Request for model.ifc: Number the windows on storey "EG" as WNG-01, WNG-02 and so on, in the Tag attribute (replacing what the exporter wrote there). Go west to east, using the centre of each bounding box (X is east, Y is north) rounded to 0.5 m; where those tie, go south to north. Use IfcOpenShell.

First a look at what the model holds.

```python
import ifcopenshell
import ifcopenshell.util.element
import ifcopenshell.util.placement

model = ifcopenshell.open("model.ifc")
print(model.schema)
storey = next(s for s in model.by_type("IfcBuildingStorey") if s.Name == "EG")
windows = [e for e in ifcopenshell.util.element.get_decomposition(storey) if e.is_a("IfcWindow")]
for e in sorted(windows, key=lambda e: e.id()):
    origin = ifcopenshell.util.placement.get_local_placement(e.ObjectPlacement)[:3, 3]
    print(e.id(), e.Tag, e.Name, origin.round(2) + 0.0, sep=" | ")
```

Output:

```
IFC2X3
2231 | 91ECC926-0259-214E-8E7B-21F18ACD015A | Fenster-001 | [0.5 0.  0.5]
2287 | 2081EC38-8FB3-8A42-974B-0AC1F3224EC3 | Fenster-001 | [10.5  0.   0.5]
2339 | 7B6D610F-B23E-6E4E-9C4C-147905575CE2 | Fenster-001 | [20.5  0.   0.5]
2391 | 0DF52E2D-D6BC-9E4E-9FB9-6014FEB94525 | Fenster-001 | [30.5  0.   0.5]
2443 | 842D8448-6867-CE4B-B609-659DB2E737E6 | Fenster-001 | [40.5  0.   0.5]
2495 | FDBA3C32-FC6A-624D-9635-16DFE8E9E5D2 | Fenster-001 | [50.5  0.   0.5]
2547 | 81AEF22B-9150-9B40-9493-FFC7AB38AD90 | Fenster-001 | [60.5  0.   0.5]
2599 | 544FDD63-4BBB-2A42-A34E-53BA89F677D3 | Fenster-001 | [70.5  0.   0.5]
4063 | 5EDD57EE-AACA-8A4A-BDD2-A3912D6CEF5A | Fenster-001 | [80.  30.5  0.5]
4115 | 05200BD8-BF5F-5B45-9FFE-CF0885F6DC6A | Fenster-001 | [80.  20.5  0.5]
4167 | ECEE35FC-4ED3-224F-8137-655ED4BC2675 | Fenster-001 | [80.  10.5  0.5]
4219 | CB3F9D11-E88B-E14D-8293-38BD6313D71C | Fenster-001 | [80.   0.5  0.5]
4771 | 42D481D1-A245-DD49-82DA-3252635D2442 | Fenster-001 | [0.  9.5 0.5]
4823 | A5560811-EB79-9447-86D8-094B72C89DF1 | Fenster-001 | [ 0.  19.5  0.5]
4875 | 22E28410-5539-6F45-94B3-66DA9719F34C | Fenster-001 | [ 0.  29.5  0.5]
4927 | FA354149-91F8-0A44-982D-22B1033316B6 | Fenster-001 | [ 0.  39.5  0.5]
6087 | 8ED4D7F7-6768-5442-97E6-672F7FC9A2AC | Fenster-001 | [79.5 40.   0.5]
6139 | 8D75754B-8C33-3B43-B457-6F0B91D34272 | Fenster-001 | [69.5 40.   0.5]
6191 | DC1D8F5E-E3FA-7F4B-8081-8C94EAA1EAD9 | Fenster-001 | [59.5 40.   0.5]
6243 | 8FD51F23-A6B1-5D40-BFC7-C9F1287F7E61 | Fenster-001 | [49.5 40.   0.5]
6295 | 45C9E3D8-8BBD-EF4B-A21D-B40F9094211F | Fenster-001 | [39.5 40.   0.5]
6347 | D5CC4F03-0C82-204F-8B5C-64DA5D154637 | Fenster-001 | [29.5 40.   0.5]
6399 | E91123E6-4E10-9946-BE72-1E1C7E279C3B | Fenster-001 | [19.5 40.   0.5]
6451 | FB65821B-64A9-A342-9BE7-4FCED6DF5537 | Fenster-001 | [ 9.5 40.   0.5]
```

```python
import ifcopenshell
import ifcopenshell.geom
import ifcopenshell.util.element
import ifcopenshell.util.shape

model = ifcopenshell.open("model.ifc")
settings = ifcopenshell.geom.settings()
settings.set("use-world-coords", True)


def centre(element):
    shape = ifcopenshell.geom.create_shape(settings, element)
    return ifcopenshell.util.shape.get_bbox_centroid(shape.geometry)


storey = next(s for s in model.by_type("IfcBuildingStorey") if s.Name == "EG")
windows = [e for e in ifcopenshell.util.element.get_decomposition(storey) if e.is_a("IfcWindow")]

# Insertion points can sit at a corner or the storey origin, so sort by the geometry (in metres).
centres = {e: centre(e) for e in windows}
windows.sort(key=lambda e: (round(centres[e][0] / 0.5), centres[e][1]))

for i, e in enumerate(windows, start=1):
    number = f"WNG-{i:02d}"
    e.Tag = number
    print(e.id(), number)

model.write("model_v2.ifc")
```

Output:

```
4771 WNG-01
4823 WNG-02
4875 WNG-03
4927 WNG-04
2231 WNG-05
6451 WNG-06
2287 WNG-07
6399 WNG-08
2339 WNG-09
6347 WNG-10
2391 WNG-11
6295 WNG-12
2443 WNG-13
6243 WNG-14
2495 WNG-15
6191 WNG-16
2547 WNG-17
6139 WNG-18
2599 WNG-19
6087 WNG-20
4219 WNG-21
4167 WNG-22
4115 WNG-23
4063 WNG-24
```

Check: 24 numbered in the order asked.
